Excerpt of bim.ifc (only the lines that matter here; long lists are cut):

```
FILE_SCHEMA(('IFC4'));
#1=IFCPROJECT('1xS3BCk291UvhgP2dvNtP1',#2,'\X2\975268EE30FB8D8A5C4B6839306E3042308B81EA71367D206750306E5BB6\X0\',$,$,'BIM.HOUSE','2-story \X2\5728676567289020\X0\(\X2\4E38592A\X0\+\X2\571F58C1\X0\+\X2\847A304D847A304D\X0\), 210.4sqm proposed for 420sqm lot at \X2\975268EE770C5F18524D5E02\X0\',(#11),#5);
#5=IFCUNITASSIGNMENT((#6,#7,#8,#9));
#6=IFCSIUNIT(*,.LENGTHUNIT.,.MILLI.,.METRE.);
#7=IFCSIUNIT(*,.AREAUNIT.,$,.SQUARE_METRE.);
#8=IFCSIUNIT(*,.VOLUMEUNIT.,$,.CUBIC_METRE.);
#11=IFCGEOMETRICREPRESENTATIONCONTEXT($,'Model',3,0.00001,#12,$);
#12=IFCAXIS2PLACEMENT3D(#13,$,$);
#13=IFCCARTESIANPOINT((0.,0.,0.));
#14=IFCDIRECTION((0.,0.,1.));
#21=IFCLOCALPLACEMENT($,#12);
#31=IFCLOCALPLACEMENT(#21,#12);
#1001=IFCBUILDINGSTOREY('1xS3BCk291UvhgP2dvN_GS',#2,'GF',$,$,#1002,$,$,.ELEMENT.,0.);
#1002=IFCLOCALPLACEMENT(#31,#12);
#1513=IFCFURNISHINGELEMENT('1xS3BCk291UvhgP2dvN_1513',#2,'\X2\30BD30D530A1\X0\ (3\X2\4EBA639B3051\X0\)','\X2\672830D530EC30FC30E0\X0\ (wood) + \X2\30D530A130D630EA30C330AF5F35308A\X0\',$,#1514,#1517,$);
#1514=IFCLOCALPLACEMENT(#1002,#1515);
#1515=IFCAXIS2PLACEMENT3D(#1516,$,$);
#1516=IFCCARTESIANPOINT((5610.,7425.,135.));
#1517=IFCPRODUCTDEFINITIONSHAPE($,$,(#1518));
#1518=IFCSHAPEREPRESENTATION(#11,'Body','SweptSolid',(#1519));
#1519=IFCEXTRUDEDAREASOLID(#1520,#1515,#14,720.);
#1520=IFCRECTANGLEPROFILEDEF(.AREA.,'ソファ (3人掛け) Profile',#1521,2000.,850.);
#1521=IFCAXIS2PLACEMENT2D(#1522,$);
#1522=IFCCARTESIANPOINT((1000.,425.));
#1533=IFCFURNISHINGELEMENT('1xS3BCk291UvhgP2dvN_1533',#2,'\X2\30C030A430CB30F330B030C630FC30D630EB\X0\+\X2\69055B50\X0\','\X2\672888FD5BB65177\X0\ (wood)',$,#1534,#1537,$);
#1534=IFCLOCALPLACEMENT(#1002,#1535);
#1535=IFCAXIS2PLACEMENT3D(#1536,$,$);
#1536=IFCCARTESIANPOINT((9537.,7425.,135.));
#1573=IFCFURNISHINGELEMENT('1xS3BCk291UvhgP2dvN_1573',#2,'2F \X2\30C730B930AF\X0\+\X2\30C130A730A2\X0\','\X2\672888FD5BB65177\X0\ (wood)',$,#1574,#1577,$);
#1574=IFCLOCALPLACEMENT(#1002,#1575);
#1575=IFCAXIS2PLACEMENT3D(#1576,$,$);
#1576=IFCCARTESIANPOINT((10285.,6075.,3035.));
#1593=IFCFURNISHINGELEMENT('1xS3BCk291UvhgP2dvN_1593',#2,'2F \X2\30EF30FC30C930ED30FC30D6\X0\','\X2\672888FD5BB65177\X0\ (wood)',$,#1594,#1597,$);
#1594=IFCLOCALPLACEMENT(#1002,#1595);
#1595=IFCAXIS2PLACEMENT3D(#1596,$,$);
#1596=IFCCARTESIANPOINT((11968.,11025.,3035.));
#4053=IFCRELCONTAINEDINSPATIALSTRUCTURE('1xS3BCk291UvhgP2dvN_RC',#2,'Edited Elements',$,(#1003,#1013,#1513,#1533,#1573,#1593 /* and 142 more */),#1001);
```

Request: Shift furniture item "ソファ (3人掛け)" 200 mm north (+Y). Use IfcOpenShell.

```python
import ifcopenshell
import ifcopenshell.api.geometry
import ifcopenshell.util.placement
import ifcopenshell.util.unit

model = ifcopenshell.open("bim.ifc")
unit_scale = ifcopenshell.util.unit.calculate_unit_scale(model)

item = model.by_id(1513)
matrix = ifcopenshell.util.placement.get_local_placement(item.ObjectPlacement)
matrix[1, 3] += 0.2 / unit_scale
ifcopenshell.api.geometry.edit_object_placement(model, product=item, matrix=matrix, is_si=False)

print(ifcopenshell.util.placement.get_local_placement(item.ObjectPlacement).round(3) + 0.0)

model.write("bim_updated.ifc")
```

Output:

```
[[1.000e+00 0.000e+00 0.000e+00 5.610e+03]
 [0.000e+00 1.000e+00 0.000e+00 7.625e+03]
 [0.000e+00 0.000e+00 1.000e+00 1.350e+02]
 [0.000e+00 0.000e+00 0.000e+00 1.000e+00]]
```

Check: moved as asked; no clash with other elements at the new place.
